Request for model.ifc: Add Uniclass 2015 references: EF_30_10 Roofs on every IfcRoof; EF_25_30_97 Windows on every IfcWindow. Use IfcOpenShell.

First a look at what the model holds.

```python
import ifcopenshell

model = ifcopenshell.open("model.ifc")
print(model.schema)
print("classifications:", [c.Name for c in model.by_type("IfcClassification")])
for ifc_class in ("IfcDoor", "IfcRoof", "IfcStair", "IfcWall", "IfcWindow"):
    print(ifc_class, len(model.by_type(ifc_class)))
```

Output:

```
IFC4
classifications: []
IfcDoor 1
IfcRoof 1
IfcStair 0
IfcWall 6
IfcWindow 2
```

```python
import ifcopenshell
import ifcopenshell.api.classification

model = ifcopenshell.open("model.ifc")

system = ifcopenshell.api.classification.add_classification(model, classification="Uniclass 2015")

codes = {
    "IfcRoof": ("EF_30_10", "Roofs"),
    "IfcWindow": ("EF_25_30_97", "Windows"),
}
for ifc_class, (code, name) in codes.items():
    products = model.by_type(ifc_class)
    ifcopenshell.api.classification.add_reference(
        model, products=products, classification=system, identification=code, name=name
    )
    print(code, len(products))

model.write("model_v2.ifc")
```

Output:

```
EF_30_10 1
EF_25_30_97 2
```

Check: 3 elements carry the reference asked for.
